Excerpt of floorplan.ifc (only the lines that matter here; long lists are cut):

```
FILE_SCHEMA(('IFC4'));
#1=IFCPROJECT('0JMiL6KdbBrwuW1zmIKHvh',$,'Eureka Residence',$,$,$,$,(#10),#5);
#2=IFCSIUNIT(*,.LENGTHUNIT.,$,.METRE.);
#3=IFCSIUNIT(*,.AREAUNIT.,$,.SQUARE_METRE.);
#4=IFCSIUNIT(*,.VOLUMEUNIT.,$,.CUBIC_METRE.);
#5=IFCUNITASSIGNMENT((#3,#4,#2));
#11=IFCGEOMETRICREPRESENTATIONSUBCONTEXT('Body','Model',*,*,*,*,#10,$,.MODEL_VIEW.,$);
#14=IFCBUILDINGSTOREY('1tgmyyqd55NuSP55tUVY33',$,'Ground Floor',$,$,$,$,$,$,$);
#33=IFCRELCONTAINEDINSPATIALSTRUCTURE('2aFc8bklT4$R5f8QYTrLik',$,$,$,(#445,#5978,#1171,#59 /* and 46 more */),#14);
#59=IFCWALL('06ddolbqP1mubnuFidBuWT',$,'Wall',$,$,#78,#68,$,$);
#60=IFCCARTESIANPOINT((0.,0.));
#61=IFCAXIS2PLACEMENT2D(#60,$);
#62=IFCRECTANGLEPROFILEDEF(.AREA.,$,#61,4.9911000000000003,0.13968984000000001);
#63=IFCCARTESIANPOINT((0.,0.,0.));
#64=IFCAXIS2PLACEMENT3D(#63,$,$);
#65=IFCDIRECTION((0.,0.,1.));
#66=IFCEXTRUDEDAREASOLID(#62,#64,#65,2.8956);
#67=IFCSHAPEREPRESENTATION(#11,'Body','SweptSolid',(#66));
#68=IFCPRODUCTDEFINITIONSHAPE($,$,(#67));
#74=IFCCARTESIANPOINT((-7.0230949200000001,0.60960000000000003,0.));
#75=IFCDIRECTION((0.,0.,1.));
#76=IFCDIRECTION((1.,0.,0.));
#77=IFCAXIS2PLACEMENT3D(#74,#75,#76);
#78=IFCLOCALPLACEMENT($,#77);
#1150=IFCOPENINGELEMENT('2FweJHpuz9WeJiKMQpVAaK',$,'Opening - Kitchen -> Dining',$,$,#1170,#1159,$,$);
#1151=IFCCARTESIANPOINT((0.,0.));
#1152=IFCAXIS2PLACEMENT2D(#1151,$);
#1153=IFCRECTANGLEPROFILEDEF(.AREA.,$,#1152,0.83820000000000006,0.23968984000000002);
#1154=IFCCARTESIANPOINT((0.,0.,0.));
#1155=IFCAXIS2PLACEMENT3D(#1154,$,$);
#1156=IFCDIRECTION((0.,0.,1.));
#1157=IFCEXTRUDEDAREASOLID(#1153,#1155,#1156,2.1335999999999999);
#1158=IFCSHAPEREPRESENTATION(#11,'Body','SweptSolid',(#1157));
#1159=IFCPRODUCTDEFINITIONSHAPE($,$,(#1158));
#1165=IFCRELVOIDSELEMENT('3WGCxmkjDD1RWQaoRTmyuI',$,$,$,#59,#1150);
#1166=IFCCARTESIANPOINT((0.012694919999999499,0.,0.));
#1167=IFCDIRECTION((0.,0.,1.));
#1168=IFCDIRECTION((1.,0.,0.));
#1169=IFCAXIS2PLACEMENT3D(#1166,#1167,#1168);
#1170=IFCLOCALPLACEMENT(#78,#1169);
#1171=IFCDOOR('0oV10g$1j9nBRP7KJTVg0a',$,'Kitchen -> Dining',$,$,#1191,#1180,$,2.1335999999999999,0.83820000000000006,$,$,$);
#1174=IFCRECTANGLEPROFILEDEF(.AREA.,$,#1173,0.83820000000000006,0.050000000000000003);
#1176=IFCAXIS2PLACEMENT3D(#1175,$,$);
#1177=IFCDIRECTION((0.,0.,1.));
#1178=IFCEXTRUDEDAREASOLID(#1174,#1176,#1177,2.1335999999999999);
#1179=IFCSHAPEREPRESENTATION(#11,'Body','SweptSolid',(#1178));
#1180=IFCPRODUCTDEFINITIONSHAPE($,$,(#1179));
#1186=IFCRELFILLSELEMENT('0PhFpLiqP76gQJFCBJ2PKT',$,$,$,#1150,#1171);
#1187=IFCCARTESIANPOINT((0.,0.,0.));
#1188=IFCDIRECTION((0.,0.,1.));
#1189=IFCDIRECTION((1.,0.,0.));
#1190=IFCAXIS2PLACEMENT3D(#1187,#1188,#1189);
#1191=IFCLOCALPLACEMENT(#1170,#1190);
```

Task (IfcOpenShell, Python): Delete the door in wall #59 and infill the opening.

```python
import ifcopenshell
import ifcopenshell.api.feature
import ifcopenshell.api.root
import ifcopenshell.geom
import ifcopenshell.util.shape

model = ifcopenshell.open("floorplan.ifc")
settings = ifcopenshell.geom.settings()


def volume(element):
    """Net volume in cubic metres, openings subtracted."""
    shape = ifcopenshell.geom.create_shape(settings, element)
    return ifcopenshell.util.shape.get_volume(shape.geometry)


door = model.by_guid("0oV10g$1j9nBRP7KJTVg0a")
opening = door.FillsVoids[0].RelatingOpeningElement
wall = opening.VoidsElements[0].RelatingBuildingElement
before = volume(wall)

ifcopenshell.api.root.remove_product(model, product=door)
ifcopenshell.api.feature.remove_feature(model, feature=opening)

after = volume(wall)

print(f"wall volume {before:.3f} -> {after:.3f} m3")

model.write("floorplan_updated.ifc")
```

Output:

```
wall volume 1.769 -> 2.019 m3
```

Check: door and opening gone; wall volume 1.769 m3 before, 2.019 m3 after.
